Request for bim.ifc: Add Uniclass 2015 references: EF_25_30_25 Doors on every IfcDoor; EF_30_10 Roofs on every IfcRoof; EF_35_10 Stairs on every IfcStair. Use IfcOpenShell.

First a look at what the model holds.

```python
import ifcopenshell

model = ifcopenshell.open("bim.ifc")
print(model.schema)
print("classifications:", [c.Name for c in model.by_type("IfcClassification")])
for ifc_class in ("IfcDoor", "IfcRoof", "IfcStair", "IfcWall", "IfcWindow"):
    print(ifc_class, len(model.by_type(ifc_class)))
```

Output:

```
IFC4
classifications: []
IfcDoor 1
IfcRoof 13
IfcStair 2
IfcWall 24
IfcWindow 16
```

```python
import ifcopenshell
import ifcopenshell.api.classification

model = ifcopenshell.open("bim.ifc")

system = ifcopenshell.api.classification.add_classification(model, classification="Uniclass 2015")

codes = {
    "IfcDoor": ("EF_25_30_25", "Doors"),
    "IfcRoof": ("EF_30_10", "Roofs"),
    "IfcStair": ("EF_35_10", "Stairs"),
}
for ifc_class, (code, name) in codes.items():
    products = model.by_type(ifc_class)
    ifcopenshell.api.classification.add_reference(
        model, products=products, classification=system, identification=code, name=name
    )
    print(code, len(products))

model.write("bim_rev.ifc")
```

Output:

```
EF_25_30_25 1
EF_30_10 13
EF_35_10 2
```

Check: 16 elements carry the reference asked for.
